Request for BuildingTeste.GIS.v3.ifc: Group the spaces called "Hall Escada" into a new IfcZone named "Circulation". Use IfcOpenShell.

First a look at what the model holds.

```python
import ifcopenshell

model = ifcopenshell.open("BuildingTeste.GIS.v3.ifc")
print(model.schema)
seen = {}
for space in model.by_type("IfcSpace"):
    seen[space.LongName] = seen.get(space.LongName, 0) + 1
for name, count in sorted(seen.items(), key=str):
    print(count, "x", name)
print("zones:", [z.Name for z in model.by_type("IfcZone")][:20])
```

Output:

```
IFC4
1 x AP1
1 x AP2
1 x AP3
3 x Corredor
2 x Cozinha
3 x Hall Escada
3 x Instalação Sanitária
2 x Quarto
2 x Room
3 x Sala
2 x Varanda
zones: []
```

```python
import ifcopenshell
import ifcopenshell.api.group
import ifcopenshell.api.root

model = ifcopenshell.open("BuildingTeste.GIS.v3.ifc")

names = {"Hall Escada"}
spaces = [s for s in model.by_type("IfcSpace") if s.LongName in names]

zone = ifcopenshell.api.root.create_entity(model, ifc_class="IfcZone", name="Circulation")
ifcopenshell.api.group.assign_group(model, products=spaces, group=zone)
print(len(spaces), "spaces in", zone.Name)

model.write("BuildingTeste.GIS.v3_rev.ifc")
```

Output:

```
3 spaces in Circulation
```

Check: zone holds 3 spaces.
